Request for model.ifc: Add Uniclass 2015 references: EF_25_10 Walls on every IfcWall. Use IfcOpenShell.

First a look at what the model holds.

```python
import ifcopenshell

model = ifcopenshell.open("model.ifc")
print(model.schema)
print("classifications:", [c.Name for c in model.by_type("IfcClassification")])
for ifc_class in ("IfcDoor", "IfcRoof", "IfcStair", "IfcWall", "IfcWindow"):
    print(ifc_class, len(model.by_type(ifc_class)))
```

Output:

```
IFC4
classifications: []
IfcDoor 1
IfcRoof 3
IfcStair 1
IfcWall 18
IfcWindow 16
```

```python
import ifcopenshell
import ifcopenshell.api.classification

model = ifcopenshell.open("model.ifc")

system = ifcopenshell.api.classification.add_classification(model, classification="Uniclass 2015")

codes = {
    "IfcWall": ("EF_25_10", "Walls"),
}
for ifc_class, (code, name) in codes.items():
    products = model.by_type(ifc_class)
    ifcopenshell.api.classification.add_reference(
        model, products=products, classification=system, identification=code, name=name
    )
    print(code, len(products))

model.write("model_rev.ifc")
```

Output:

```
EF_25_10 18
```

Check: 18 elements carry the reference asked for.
